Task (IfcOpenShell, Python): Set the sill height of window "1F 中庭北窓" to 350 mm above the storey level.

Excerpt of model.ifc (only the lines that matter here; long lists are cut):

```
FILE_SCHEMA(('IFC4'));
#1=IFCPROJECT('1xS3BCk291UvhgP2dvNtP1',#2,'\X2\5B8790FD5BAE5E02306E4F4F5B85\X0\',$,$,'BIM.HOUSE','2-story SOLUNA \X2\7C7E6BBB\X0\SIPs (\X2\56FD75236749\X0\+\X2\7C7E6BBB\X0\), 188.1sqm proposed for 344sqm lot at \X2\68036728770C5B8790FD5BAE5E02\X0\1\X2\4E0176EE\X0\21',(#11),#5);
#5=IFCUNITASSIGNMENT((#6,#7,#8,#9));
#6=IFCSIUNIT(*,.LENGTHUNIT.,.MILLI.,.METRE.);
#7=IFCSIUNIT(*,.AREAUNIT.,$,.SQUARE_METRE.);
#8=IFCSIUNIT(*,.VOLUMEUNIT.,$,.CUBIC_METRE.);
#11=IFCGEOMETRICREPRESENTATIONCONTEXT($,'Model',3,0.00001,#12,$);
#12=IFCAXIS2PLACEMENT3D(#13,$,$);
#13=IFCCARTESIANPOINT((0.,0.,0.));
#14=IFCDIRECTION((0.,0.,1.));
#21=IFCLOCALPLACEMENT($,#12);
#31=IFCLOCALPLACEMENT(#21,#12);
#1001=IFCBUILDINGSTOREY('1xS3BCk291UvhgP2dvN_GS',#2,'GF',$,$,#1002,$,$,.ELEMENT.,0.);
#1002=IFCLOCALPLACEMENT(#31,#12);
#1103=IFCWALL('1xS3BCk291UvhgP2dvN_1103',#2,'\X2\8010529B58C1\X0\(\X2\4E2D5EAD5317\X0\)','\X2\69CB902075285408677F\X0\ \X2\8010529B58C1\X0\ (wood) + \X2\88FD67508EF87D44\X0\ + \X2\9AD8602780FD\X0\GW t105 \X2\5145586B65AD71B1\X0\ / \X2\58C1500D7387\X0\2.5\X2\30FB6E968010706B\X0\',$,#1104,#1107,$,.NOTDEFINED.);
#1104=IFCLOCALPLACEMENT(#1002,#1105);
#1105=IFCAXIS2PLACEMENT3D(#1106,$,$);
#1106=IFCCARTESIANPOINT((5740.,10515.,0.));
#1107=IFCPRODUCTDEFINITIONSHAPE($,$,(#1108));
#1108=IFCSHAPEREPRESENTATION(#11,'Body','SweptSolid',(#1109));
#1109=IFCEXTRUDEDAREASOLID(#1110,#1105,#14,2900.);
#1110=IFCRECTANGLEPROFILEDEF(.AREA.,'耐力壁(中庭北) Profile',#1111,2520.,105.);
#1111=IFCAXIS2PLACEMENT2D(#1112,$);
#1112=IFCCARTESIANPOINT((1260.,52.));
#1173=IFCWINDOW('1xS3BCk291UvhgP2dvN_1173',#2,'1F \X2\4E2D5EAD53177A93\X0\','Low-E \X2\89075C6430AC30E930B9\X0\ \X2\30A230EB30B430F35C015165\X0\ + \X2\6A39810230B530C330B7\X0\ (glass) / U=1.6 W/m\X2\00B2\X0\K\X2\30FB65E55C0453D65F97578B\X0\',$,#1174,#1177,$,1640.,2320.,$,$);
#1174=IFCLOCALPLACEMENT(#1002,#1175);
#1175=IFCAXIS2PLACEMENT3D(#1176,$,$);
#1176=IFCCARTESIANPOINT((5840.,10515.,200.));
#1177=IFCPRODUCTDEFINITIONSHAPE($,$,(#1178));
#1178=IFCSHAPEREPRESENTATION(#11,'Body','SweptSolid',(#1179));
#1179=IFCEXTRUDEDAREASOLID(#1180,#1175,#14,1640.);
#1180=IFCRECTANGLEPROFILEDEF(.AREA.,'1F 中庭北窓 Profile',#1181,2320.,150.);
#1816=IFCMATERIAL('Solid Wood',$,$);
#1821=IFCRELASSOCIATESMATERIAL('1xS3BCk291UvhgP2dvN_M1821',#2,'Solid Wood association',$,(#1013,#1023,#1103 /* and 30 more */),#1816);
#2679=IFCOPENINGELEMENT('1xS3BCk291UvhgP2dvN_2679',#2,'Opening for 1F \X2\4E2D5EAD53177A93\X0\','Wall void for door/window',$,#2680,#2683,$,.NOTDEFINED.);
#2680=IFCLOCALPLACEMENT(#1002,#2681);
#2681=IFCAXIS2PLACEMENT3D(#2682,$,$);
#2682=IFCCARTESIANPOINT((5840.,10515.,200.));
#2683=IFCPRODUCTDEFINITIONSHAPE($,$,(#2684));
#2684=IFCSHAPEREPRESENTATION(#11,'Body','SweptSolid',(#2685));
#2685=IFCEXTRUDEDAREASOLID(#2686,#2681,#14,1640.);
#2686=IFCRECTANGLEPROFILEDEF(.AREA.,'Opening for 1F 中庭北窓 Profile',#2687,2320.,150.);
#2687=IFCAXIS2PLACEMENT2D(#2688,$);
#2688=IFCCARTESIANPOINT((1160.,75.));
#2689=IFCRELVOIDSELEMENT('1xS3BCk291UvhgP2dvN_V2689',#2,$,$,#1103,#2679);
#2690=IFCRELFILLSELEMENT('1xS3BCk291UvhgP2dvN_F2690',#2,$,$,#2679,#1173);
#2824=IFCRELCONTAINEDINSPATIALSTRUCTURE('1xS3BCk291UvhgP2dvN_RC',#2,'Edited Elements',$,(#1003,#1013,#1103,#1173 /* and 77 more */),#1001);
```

```python
import numpy as np
import ifcopenshell
import ifcopenshell.api.geometry
import ifcopenshell.geom
import ifcopenshell.util.element
import ifcopenshell.util.placement
import ifcopenshell.util.shape
import ifcopenshell.util.unit

model = ifcopenshell.open("model.ifc")
unit_scale = ifcopenshell.util.unit.calculate_unit_scale(model)

window = model.by_guid("1xS3BCk291UvhgP2dvN_1173")
opening = window.FillsVoids[0].RelatingOpeningElement
storey = ifcopenshell.util.element.get_container(window, ifc_class="IfcBuildingStorey")
level = ifcopenshell.util.placement.get_local_placement(storey.ObjectPlacement)[2, 3]

# The opening's origin need not be at the sill, so measure its lowest point.
shape = ifcopenshell.geom.create_shape(ifcopenshell.geom.settings(), opening)
bottom = ifcopenshell.util.shape.get_shape_bottom_elevation(shape, shape.geometry) / unit_scale
dz = level + 350.0 - bottom

shift = np.array([0.0, 0.0, dz])
# The window is not placed relative to its opening, so move both.
for product in (opening, window):
    matrix = ifcopenshell.util.placement.get_local_placement(product.ObjectPlacement)
    matrix[:3, 3] += shift
    ifcopenshell.api.geometry.edit_object_placement(model, product=product, matrix=matrix, is_si=False)

print(f"moved by {dz * unit_scale:+.3f} m")

model.write("model_v2.ifc")
```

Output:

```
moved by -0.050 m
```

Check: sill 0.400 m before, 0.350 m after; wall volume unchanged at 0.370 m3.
